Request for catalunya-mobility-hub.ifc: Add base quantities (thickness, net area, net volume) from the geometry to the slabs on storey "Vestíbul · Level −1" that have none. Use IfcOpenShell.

First a look at what the model holds.

```python
import ifcopenshell
import ifcopenshell.util.element
import ifcopenshell.util.unit

model = ifcopenshell.open("catalunya-mobility-hub.ifc")
print(model.schema)
for unit_type in ("LENGTHUNIT", "AREAUNIT", "VOLUMEUNIT"):
    print(unit_type, ifcopenshell.util.unit.calculate_unit_scale(model, unit_type))
storey = next(s for s in model.by_type("IfcBuildingStorey") if s.Name == "Vestíbul · Level −1")
slabs = [e for e in ifcopenshell.util.element.get_decomposition(storey) if e.is_a("IfcSlab")]
for e in sorted(slabs, key=lambda e: e.id()):
    print(e.id(), e.is_a(), e.Name, list(ifcopenshell.util.element.get_psets(e, qtos_only=True)), sep=" | ")
```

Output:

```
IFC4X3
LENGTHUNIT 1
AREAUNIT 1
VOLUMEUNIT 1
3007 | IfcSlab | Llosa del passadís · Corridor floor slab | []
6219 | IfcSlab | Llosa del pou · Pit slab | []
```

```python
import ifcopenshell
import ifcopenshell.api.pset
import ifcopenshell.geom
import ifcopenshell.util.element
import ifcopenshell.util.shape
import ifcopenshell.util.unit

model = ifcopenshell.open("catalunya-mobility-hub.ifc")
unit_scale = ifcopenshell.util.unit.calculate_unit_scale(model)
area_scale = ifcopenshell.util.unit.calculate_unit_scale(model, "AREAUNIT")
volume_scale = ifcopenshell.util.unit.calculate_unit_scale(model, "VOLUMEUNIT")
settings = ifcopenshell.geom.settings()

storey = next(s for s in model.by_type("IfcBuildingStorey") if s.Name == "Vestíbul · Level −1")
slabs = [e for e in ifcopenshell.util.element.get_decomposition(storey) if e.is_a("IfcSlab")]

for e in sorted(slabs, key=lambda e: e.id()):
    if ifcopenshell.util.element.get_psets(e, qtos_only=True, should_inherit=False):
        continue
    # Geometry comes back in metres, in the element's own axes.
    shape = ifcopenshell.geom.create_shape(settings, e)
    values = {
        "Width": ifcopenshell.util.shape.get_z(shape.geometry) / unit_scale,
        "NetArea": ifcopenshell.util.shape.get_footprint_area(shape.geometry) / area_scale,
        "NetVolume": ifcopenshell.util.shape.get_volume(shape.geometry) / volume_scale,
    }
    qto = ifcopenshell.api.pset.add_qto(model, product=e, name="Qto_SlabBaseQuantities")
    ifcopenshell.api.pset.edit_qto(model, qto=qto, properties=values)
    print(e.id(), {k: round(v, 3) for k, v in values.items()})

model.write("catalunya-mobility-hub_v2.ifc")
```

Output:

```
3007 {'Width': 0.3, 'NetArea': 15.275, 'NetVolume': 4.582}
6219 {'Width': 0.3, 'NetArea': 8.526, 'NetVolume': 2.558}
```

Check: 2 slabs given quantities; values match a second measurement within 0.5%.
